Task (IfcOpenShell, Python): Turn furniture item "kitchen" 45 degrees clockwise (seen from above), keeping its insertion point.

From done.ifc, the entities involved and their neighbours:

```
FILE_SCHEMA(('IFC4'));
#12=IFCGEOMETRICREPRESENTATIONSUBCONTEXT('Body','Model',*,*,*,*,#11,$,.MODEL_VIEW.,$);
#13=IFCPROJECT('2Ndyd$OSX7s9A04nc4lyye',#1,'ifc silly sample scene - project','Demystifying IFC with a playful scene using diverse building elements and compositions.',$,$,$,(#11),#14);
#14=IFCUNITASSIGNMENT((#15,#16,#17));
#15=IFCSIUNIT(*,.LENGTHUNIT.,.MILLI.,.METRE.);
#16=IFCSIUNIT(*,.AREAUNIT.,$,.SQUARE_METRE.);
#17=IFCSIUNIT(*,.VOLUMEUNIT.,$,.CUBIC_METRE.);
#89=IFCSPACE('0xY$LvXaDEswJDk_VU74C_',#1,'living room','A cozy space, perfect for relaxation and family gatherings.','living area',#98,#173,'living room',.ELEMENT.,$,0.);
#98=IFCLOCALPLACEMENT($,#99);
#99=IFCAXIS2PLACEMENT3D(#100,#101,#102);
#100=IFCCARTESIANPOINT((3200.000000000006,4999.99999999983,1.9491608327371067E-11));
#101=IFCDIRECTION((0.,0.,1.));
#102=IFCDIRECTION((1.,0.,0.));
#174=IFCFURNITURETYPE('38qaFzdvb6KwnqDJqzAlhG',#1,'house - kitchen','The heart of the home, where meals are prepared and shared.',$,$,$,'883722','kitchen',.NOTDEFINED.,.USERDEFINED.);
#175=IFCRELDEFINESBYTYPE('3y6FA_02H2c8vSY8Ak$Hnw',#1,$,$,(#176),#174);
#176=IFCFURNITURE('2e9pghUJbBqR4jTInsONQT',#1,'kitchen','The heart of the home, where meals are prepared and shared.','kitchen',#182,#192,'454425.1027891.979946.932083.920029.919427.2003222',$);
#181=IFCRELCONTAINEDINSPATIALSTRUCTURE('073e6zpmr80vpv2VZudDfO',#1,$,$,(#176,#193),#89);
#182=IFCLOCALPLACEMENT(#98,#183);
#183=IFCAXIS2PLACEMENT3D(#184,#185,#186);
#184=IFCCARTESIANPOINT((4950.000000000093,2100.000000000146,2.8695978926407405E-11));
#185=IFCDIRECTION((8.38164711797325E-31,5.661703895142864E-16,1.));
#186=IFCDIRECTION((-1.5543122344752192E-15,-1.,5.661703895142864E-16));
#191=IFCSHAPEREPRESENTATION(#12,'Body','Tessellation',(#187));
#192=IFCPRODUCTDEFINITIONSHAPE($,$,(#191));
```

```python
import ifcopenshell
import ifcopenshell.api.geometry
import ifcopenshell.util.placement

model = ifcopenshell.open("done.ifc")

item = model.by_guid("2e9pghUJbBqR4jTInsONQT")
matrix = ifcopenshell.util.placement.get_local_placement(item.ObjectPlacement)
matrix = matrix @ ifcopenshell.util.placement.rotation(-45, "Z")
ifcopenshell.api.geometry.edit_object_placement(model, product=item, matrix=matrix, is_si=False)

print(ifcopenshell.util.placement.get_local_placement(item.ObjectPlacement).round(3) + 0.0)

model.write("done_v2.ifc")
```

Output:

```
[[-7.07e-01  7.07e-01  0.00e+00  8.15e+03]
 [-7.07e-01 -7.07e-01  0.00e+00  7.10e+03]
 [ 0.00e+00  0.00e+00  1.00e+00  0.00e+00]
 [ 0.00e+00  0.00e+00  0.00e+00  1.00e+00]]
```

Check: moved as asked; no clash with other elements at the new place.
